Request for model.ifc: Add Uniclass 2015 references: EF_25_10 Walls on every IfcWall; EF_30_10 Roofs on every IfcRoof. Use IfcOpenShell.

First a look at what the model holds.

```python
import ifcopenshell

model = ifcopenshell.open("model.ifc")
print(model.schema)
print("classifications:", [c.Name for c in model.by_type("IfcClassification")])
for ifc_class in ("IfcDoor", "IfcRoof", "IfcStair", "IfcWall", "IfcWindow"):
    print(ifc_class, len(model.by_type(ifc_class)))
```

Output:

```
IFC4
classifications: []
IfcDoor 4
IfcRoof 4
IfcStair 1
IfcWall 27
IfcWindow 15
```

```python
import ifcopenshell
import ifcopenshell.api.classification

model = ifcopenshell.open("model.ifc")

system = ifcopenshell.api.classification.add_classification(model, classification="Uniclass 2015")

codes = {
    "IfcWall": ("EF_25_10", "Walls"),
    "IfcRoof": ("EF_30_10", "Roofs"),
}
for ifc_class, (code, name) in codes.items():
    products = model.by_type(ifc_class)
    ifcopenshell.api.classification.add_reference(
        model, products=products, classification=system, identification=code, name=name
    )
    print(code, len(products))

model.write("model_edited.ifc")
```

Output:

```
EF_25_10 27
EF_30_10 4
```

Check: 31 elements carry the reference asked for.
